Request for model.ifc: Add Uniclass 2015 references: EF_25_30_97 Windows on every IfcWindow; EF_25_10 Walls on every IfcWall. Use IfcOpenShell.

First a look at what the model holds.

```python
import ifcopenshell

model = ifcopenshell.open("model.ifc")
print(model.schema)
print("classifications:", [c.Name for c in model.by_type("IfcClassification")])
for ifc_class in ("IfcDoor", "IfcRoof", "IfcStair", "IfcWall", "IfcWindow"):
    print(ifc_class, len(model.by_type(ifc_class)))
```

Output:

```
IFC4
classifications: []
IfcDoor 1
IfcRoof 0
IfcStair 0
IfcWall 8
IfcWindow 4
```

```python
import ifcopenshell
import ifcopenshell.api.classification

model = ifcopenshell.open("model.ifc")

system = ifcopenshell.api.classification.add_classification(model, classification="Uniclass 2015")

codes = {
    "IfcWindow": ("EF_25_30_97", "Windows"),
    "IfcWall": ("EF_25_10", "Walls"),
}
for ifc_class, (code, name) in codes.items():
    products = model.by_type(ifc_class)
    ifcopenshell.api.classification.add_reference(
        model, products=products, classification=system, identification=code, name=name
    )
    print(code, len(products))

model.write("model-out.ifc")
```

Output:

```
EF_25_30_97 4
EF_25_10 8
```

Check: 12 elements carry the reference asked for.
